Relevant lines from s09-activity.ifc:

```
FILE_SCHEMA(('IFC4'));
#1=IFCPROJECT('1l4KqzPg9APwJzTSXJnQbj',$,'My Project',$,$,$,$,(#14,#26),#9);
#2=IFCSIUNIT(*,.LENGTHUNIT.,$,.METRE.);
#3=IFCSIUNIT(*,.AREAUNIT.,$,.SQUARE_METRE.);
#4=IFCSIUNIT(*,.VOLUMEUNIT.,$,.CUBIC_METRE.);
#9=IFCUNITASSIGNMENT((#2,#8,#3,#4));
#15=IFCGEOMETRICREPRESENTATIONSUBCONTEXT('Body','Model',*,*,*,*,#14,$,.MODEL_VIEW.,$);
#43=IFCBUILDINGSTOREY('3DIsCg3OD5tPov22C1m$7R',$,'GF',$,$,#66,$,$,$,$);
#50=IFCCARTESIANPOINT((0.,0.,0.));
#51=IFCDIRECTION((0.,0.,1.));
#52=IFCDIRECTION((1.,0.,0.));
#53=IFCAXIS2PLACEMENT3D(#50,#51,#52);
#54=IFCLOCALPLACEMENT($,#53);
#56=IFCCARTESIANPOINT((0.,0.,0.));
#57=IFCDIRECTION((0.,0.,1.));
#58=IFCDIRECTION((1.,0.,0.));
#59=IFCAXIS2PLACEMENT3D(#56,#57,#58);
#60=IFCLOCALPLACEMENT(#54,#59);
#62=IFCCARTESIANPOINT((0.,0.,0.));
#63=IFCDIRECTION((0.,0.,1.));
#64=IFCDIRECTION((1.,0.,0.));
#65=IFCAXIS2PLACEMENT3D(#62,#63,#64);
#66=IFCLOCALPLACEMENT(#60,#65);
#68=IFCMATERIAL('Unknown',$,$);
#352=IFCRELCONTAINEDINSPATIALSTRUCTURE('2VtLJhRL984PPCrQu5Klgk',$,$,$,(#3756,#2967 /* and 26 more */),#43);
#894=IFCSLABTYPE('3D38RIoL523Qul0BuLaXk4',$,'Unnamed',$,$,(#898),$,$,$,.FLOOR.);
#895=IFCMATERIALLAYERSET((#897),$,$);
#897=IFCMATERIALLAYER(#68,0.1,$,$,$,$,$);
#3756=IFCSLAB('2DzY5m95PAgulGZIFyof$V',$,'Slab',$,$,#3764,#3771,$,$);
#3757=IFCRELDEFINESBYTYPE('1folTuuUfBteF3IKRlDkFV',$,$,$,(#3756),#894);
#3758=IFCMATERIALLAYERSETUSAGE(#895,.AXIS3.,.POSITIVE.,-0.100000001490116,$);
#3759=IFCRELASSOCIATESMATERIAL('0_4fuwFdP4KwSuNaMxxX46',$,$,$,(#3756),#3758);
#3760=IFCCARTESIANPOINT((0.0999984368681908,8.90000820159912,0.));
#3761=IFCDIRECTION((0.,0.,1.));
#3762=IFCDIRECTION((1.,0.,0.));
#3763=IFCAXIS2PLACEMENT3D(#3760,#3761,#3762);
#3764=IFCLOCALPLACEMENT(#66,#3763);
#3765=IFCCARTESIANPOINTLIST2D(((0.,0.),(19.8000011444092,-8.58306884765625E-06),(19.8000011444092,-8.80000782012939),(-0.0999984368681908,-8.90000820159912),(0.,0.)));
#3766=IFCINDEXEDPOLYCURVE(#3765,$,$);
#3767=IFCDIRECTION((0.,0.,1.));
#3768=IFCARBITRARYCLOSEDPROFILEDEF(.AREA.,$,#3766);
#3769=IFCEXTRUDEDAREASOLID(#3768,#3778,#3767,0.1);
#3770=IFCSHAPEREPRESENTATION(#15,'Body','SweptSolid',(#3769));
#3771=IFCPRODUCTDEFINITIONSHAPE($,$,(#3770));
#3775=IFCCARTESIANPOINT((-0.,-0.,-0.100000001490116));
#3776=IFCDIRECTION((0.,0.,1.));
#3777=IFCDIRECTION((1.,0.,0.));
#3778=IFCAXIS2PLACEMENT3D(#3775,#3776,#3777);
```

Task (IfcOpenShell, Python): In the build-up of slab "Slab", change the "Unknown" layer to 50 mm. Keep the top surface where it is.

```python
import ifcopenshell
import ifcopenshell.util.element
import ifcopenshell.util.representation
import ifcopenshell.util.unit

model = ifcopenshell.open("s09-activity.ifc")
unit_scale = ifcopenshell.util.unit.calculate_unit_scale(model)

layer_set = model.by_id(895)
layer = next(l for l in layer_set.MaterialLayers if l.Material and l.Material.Name == "Unknown")
change = 0.05 / unit_scale - layer.LayerThickness
layer.LayerThickness += change

# Geometry does not follow the layer set by itself.
slabs = [e for e in ifcopenshell.util.element.get_elements_by_material(model, layer_set) if e.is_a("IfcSlab")]
for slab in sorted(slabs, key=lambda e: e.id()):
    body = ifcopenshell.util.representation.get_representation(slab, "Model", "Body")
    solid = body.Items[0]
    old_depth = solid.Depth
    solid.Depth += change
    # Extruded upwards: lower the start of the extrusion so the top stays.
    x, y, z = solid.Position.Location.Coordinates
    solid.Position.Location = model.createIfcCartesianPoint((x, y, z - change))
    print(slab.id(), f"{old_depth:g} -> {solid.Depth:g}")

# The layers are counted up from the underside, which has moved.
for usage in {ifcopenshell.util.element.get_material(slab) for slab in slabs}:
    usage.OffsetFromReferenceLine -= change

model.write("s09-activity_v2.ifc")
```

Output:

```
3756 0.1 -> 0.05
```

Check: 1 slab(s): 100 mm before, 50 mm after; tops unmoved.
